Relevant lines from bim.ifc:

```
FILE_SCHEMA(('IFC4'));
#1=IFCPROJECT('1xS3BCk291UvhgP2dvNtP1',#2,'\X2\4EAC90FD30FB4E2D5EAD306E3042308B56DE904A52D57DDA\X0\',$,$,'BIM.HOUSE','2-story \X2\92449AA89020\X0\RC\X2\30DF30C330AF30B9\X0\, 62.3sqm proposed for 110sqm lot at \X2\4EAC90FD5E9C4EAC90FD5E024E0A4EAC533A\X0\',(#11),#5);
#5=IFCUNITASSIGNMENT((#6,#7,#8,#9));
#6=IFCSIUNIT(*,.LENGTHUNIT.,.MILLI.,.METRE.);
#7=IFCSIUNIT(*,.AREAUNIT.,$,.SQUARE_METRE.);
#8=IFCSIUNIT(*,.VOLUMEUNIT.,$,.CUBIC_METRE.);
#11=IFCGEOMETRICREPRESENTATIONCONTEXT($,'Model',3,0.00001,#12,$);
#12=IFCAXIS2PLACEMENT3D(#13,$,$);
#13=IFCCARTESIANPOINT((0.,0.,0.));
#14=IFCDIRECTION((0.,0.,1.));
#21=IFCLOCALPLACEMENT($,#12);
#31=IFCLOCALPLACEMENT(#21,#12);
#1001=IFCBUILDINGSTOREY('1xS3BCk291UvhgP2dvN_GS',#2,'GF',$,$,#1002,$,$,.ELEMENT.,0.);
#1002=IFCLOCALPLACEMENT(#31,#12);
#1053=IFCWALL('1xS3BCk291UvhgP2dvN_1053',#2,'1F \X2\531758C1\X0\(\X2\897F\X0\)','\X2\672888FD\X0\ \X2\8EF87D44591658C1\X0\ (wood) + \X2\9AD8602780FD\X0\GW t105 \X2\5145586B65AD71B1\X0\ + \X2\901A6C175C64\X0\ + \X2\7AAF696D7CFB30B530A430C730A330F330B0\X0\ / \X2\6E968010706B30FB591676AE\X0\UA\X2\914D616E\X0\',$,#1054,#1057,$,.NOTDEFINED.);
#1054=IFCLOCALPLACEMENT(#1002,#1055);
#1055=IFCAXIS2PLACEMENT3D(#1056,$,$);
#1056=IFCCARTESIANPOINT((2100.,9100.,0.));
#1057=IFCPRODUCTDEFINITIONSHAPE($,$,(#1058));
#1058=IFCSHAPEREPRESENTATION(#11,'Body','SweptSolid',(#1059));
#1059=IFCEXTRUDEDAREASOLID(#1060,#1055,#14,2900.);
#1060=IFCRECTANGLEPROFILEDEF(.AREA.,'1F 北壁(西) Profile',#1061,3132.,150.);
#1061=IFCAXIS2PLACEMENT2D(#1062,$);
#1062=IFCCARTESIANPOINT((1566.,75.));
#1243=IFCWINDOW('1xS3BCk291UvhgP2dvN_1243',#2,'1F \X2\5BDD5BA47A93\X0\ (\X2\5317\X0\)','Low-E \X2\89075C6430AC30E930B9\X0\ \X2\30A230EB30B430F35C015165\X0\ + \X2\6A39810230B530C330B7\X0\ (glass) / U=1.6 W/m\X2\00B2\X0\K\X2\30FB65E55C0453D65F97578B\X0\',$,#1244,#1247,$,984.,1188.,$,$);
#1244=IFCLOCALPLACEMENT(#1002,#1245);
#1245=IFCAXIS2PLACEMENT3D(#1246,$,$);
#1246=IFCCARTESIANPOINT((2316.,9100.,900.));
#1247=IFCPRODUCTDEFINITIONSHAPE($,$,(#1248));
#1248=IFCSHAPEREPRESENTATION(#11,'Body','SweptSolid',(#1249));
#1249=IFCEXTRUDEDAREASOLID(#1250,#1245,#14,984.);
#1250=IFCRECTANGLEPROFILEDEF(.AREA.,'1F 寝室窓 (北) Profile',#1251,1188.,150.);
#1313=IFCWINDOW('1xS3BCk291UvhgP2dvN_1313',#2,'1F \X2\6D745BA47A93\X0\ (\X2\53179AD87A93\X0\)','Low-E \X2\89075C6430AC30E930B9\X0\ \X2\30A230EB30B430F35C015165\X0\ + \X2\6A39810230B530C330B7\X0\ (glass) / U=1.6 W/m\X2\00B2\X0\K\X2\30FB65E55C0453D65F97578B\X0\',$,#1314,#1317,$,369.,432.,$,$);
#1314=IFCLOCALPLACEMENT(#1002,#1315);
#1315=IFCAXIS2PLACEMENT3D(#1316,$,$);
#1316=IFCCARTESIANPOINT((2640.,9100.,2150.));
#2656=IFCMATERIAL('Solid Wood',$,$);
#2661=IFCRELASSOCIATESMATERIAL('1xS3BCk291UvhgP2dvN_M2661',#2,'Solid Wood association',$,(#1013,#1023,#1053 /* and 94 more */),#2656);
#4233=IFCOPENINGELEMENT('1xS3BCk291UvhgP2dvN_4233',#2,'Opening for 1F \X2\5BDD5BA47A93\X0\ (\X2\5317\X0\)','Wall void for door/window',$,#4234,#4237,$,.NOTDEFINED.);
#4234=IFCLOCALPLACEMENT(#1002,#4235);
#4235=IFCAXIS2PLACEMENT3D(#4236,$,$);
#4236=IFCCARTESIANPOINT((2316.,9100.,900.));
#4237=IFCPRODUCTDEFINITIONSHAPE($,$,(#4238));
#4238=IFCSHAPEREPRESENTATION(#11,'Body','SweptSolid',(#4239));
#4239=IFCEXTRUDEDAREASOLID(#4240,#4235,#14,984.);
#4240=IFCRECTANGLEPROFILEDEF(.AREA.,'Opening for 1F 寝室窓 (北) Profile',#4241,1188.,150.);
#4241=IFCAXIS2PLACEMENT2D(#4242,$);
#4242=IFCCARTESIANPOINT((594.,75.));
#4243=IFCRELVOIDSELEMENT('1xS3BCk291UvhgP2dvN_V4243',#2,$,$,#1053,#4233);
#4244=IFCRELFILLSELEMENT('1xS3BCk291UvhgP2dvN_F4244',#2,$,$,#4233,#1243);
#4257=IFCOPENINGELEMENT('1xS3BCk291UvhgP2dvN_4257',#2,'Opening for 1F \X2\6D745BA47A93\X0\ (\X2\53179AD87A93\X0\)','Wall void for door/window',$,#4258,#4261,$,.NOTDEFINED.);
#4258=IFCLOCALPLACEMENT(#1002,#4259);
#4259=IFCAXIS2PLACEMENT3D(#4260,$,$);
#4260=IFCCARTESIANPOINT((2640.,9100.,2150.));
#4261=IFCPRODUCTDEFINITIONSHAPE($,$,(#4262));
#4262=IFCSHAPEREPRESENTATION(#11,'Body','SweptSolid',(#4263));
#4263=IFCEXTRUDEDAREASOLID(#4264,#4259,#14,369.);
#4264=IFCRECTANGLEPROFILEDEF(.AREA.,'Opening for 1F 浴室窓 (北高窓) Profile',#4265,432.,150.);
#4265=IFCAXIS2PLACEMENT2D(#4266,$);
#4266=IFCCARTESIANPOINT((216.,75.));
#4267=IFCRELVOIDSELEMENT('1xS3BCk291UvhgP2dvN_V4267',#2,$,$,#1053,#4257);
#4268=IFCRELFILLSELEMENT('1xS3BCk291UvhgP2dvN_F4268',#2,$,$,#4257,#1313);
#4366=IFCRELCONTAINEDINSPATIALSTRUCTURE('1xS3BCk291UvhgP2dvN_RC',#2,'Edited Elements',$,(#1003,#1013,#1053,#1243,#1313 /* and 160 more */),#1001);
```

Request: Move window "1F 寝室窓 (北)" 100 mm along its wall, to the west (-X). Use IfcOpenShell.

```python
import ifcopenshell
import ifcopenshell.api.geometry
import ifcopenshell.util.placement
import ifcopenshell.util.unit

model = ifcopenshell.open("bim.ifc")
unit_scale = ifcopenshell.util.unit.calculate_unit_scale(model)

window = model.by_guid("1xS3BCk291UvhgP2dvN_1243")
opening = window.FillsVoids[0].RelatingOpeningElement
wall = opening.VoidsElements[0].RelatingBuildingElement

wall_matrix = ifcopenshell.util.placement.get_local_placement(wall.ObjectPlacement)
shift = wall_matrix[:3, 0] * -0.1 / unit_scale
before = ifcopenshell.util.placement.get_local_placement(window.ObjectPlacement)[:3, 3].copy()

# The window is not placed relative to its opening, so move both.
for product in (opening, window):
    matrix = ifcopenshell.util.placement.get_local_placement(product.ObjectPlacement)
    matrix[:3, 3] += shift
    ifcopenshell.api.geometry.edit_object_placement(model, product=product, matrix=matrix, is_si=False)

after = ifcopenshell.util.placement.get_local_placement(window.ObjectPlacement)[:3, 3]
print("window moved by", (after - before).round(3) + 0.0)

model.write("bim_rev.ifc")
```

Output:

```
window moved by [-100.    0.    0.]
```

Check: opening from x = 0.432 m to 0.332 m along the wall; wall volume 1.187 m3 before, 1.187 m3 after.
